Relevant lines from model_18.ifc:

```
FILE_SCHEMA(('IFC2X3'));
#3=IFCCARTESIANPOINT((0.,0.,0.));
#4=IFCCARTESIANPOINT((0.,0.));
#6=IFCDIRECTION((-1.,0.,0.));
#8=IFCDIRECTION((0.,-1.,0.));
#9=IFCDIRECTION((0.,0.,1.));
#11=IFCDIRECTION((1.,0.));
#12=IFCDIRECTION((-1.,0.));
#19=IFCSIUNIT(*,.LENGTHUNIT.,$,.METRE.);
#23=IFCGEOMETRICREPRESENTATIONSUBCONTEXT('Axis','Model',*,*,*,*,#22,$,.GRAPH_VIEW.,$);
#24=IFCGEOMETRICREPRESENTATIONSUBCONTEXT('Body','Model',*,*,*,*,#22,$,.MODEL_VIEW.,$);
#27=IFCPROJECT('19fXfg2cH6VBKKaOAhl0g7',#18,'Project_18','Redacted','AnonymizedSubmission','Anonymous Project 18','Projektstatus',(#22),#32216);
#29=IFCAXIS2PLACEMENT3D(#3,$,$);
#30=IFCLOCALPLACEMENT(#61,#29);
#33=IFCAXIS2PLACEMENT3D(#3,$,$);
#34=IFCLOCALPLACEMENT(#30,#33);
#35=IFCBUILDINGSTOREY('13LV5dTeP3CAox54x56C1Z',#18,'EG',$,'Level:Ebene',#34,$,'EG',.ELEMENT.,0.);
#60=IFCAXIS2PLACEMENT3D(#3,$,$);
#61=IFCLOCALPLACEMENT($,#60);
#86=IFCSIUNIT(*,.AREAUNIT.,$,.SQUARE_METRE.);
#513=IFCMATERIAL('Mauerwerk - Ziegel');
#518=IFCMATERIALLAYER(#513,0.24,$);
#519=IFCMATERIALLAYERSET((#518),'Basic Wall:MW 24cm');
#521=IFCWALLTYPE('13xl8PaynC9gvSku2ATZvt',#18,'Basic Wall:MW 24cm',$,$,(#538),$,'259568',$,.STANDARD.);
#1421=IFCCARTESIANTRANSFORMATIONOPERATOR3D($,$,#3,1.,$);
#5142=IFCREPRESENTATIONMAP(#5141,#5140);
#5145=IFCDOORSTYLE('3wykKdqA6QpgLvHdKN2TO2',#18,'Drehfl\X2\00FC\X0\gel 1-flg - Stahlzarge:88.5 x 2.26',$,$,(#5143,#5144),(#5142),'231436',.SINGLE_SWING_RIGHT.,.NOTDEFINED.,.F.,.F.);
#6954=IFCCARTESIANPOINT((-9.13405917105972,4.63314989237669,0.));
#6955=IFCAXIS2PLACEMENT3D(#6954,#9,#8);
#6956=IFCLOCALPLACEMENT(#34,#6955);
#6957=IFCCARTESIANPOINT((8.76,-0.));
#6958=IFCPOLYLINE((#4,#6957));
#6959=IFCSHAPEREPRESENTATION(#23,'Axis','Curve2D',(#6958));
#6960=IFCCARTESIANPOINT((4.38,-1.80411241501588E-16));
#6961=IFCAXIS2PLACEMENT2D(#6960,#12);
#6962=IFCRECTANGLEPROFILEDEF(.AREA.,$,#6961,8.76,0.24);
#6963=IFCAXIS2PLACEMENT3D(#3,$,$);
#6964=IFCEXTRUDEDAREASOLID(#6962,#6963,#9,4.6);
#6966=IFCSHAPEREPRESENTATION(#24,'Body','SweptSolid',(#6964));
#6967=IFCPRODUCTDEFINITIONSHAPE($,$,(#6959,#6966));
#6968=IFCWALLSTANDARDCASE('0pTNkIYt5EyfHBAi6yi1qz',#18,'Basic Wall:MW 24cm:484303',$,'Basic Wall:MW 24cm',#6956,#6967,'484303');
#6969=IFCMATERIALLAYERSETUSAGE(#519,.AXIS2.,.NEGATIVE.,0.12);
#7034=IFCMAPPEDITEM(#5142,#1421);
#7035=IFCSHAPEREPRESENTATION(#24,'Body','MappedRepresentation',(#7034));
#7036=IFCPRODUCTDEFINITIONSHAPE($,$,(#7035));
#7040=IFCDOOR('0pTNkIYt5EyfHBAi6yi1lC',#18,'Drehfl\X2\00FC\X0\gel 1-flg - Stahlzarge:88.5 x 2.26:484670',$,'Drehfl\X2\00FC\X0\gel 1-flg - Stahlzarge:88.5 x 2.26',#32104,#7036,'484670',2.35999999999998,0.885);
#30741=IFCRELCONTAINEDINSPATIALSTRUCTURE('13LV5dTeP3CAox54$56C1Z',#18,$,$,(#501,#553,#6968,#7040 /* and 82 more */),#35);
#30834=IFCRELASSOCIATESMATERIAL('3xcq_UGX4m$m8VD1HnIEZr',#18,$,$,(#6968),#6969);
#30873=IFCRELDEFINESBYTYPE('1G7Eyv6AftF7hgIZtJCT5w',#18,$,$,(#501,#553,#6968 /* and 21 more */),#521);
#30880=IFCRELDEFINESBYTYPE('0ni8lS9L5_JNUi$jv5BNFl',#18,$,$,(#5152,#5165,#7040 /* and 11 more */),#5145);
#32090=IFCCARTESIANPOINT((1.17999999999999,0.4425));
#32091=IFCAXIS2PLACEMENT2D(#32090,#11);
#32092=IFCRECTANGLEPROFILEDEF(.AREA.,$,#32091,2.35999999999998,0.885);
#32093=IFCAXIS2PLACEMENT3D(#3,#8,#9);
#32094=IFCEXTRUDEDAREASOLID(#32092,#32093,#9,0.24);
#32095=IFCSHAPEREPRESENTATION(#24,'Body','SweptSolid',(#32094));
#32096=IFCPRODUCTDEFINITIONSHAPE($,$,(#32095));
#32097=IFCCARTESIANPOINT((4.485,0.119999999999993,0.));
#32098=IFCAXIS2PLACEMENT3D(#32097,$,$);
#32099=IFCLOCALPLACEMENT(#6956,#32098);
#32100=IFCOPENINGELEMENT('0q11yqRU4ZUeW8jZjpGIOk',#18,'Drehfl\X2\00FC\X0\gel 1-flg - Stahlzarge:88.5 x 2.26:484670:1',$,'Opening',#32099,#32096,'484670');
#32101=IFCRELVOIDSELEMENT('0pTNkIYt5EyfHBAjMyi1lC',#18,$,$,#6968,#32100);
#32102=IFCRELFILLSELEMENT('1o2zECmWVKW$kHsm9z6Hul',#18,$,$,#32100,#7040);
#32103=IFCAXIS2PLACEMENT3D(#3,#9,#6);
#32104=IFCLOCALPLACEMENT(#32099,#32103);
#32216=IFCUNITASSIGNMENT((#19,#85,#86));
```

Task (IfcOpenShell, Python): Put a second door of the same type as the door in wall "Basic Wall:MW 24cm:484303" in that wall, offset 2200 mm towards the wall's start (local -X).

```python
import ifcopenshell
import ifcopenshell.api.feature
import ifcopenshell.api.geometry
import ifcopenshell.api.root
import ifcopenshell.geom
import ifcopenshell.util.element
import ifcopenshell.util.placement
import ifcopenshell.util.shape

model = ifcopenshell.open("model_18.ifc")
settings = ifcopenshell.geom.settings()


def volume(element):
    """Net volume in cubic metres, openings subtracted."""
    shape = ifcopenshell.geom.create_shape(settings, element)
    return ifcopenshell.util.shape.get_volume(shape.geometry)


def reuse_history(source, copy):
    """copy_class also copies each property set's owner history, people and application; keep the originals."""
    for rel in copy.IsDefinedBy:
        if rel.is_a("IfcRelDefinesByProperties") and (history := rel.RelatingPropertyDefinition.OwnerHistory):
            rel.RelatingPropertyDefinition.OwnerHistory = source.OwnerHistory
            ifcopenshell.util.element.remove_deep2(model, history)


door = model.by_guid("0pTNkIYt5EyfHBAi6yi1lC")
opening = door.FillsVoids[0].RelatingOpeningElement
wall = opening.VoidsElements[0].RelatingBuildingElement
before = volume(wall)
shift = ifcopenshell.util.placement.get_local_placement(wall.ObjectPlacement)[:3, 0] * -2.2

# copy_class copies the void relationship, type, container and properties, but no geometry.
new_opening = ifcopenshell.api.root.copy_class(model, product=opening)
new_opening.Representation = ifcopenshell.util.element.copy_deep(
    model, opening.Representation, exclude=["IfcGeometricRepresentationContext", "IfcRepresentationMap"]
)
new_opening.Name = "Drehflügel 1-flg - Stahlzarge:88.5 x 2.26"
new_opening.Tag = None
new_door = ifcopenshell.api.root.copy_class(model, product=door)
new_door.Representation = ifcopenshell.util.element.copy_deep(
    model, door.Representation, exclude=["IfcGeometricRepresentationContext", "IfcRepresentationMap"]
)
new_door.Name = "Drehflügel 1-flg - Stahlzarge:88.5 x 2.26"
new_door.Tag = None
reuse_history(door, new_door)
fills = ifcopenshell.api.feature.add_filling(model, opening=new_opening, element=new_door)
fills.OwnerHistory = new_door.OwnerHistory  # required in IFC2X3

for old, new in ((opening, new_opening), (door, new_door)):
    matrix = ifcopenshell.util.placement.get_local_placement(old.ObjectPlacement)
    matrix[:3, 3] += shift
    ifcopenshell.api.geometry.edit_object_placement(model, product=new, matrix=matrix, is_si=False)

after = volume(wall)

print(f"wall volume {before:.3f} -> {after:.3f} m3")

model.write("model_18_v2.ifc")
```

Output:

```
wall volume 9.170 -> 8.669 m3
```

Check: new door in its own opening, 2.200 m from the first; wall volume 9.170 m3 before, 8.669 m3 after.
